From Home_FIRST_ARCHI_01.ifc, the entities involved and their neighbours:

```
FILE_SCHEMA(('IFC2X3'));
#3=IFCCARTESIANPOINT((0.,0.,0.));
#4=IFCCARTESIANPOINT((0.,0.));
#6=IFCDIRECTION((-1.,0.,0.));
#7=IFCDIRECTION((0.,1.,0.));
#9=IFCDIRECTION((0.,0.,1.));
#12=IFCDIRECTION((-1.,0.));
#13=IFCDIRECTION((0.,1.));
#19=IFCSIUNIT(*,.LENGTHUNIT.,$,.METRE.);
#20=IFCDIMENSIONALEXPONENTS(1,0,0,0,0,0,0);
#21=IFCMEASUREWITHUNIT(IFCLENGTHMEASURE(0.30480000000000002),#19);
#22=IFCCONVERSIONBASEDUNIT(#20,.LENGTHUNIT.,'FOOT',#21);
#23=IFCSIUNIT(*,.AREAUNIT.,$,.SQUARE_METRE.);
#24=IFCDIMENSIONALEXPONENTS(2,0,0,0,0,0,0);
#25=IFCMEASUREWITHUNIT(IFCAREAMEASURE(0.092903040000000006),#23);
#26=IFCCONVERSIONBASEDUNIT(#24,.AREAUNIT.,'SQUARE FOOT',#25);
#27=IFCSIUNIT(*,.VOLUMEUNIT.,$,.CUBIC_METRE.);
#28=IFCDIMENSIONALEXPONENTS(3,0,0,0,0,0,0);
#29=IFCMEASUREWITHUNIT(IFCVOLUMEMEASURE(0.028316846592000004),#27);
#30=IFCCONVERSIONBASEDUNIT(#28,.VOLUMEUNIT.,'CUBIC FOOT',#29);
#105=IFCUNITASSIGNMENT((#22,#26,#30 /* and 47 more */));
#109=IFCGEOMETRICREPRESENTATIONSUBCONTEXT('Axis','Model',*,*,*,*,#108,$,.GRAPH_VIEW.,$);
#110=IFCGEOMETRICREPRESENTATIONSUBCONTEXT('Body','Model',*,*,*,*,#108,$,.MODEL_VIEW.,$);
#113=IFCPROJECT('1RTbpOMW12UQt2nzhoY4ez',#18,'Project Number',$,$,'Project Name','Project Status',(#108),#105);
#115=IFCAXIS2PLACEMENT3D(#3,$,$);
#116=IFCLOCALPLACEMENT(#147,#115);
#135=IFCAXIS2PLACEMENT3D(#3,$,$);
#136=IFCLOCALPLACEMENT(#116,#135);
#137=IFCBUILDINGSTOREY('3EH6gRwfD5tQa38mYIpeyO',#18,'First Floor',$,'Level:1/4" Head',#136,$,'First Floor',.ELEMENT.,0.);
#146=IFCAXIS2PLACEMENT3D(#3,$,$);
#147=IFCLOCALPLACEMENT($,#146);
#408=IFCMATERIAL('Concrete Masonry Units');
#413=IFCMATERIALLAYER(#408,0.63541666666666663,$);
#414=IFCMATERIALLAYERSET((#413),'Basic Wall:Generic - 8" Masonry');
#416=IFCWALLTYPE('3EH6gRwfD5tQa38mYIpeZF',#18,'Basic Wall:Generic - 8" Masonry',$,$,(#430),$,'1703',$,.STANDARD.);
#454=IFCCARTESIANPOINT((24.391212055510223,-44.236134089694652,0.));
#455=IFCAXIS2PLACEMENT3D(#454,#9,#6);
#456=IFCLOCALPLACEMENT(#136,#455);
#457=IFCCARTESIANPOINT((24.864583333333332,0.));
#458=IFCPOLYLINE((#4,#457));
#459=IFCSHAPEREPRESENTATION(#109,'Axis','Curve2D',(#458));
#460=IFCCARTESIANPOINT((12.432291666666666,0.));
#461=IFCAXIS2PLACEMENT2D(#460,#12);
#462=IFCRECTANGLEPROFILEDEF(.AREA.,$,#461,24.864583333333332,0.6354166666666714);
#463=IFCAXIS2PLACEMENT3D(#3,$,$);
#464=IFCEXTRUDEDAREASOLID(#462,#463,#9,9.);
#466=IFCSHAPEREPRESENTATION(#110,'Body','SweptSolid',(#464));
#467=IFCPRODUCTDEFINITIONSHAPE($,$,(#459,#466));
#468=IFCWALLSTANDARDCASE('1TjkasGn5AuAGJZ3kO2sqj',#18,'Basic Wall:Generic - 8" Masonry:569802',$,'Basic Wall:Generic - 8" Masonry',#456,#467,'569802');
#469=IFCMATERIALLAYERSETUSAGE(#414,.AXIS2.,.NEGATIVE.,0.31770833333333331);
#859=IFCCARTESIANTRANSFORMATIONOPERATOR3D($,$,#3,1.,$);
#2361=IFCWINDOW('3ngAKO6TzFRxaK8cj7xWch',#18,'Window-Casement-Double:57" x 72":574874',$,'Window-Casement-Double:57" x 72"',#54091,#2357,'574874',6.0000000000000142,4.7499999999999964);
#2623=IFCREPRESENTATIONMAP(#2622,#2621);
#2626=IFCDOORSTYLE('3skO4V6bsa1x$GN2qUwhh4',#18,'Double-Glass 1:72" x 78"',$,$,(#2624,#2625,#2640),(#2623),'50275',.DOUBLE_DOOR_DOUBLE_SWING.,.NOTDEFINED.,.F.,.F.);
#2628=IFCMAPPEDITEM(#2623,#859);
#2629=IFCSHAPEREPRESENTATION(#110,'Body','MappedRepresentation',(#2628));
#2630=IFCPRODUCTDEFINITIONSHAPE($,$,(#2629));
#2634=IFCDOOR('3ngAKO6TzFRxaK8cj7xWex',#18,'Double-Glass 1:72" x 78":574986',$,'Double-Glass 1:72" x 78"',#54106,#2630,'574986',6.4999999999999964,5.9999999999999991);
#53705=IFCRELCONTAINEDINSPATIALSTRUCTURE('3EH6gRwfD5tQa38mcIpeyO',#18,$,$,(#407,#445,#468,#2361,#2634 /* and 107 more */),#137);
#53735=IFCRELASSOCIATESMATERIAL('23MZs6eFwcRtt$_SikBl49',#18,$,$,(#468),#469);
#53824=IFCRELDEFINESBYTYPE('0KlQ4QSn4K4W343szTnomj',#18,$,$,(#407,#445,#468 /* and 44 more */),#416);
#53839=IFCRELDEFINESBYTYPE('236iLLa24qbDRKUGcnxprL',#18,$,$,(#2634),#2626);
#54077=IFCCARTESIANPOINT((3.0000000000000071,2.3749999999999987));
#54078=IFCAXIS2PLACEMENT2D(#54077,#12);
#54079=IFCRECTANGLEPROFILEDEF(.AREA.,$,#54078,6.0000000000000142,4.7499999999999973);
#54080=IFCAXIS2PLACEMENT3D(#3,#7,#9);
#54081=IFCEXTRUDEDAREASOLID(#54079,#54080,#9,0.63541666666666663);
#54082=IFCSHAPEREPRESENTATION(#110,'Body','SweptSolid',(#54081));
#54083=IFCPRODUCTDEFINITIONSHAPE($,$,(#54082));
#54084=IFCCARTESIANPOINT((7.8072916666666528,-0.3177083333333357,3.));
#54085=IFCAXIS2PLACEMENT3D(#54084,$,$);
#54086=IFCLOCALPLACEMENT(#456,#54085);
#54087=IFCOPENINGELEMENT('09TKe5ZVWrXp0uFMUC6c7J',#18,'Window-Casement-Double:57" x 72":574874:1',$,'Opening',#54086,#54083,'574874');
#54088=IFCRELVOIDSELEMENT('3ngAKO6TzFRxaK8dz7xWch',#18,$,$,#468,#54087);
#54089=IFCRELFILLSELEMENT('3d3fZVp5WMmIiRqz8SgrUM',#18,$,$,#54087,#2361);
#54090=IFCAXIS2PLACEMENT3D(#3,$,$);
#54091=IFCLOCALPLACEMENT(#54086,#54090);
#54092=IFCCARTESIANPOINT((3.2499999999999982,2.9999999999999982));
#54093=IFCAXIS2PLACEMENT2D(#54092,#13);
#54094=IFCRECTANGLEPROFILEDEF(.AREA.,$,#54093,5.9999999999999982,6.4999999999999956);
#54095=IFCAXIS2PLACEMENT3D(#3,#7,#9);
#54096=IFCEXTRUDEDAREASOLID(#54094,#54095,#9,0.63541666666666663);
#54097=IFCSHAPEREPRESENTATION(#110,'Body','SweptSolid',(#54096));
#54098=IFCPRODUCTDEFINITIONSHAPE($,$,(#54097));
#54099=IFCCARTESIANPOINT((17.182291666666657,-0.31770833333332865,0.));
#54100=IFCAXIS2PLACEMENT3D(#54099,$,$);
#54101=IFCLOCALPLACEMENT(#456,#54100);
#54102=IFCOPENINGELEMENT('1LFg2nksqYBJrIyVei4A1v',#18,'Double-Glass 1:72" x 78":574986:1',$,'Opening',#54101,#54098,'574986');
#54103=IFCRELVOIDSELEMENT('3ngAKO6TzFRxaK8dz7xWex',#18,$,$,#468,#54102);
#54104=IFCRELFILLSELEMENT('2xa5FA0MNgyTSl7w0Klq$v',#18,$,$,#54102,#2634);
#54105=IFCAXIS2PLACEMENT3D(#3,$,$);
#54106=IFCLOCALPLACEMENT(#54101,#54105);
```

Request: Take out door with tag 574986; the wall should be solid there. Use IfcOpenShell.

```python
import ifcopenshell
import ifcopenshell.api.feature
import ifcopenshell.api.root
import ifcopenshell.geom
import ifcopenshell.util.shape

model = ifcopenshell.open("Home_FIRST_ARCHI_01.ifc")
settings = ifcopenshell.geom.settings()


def volume(element):
    """Net volume in cubic metres, openings subtracted."""
    shape = ifcopenshell.geom.create_shape(settings, element)
    return ifcopenshell.util.shape.get_volume(shape.geometry)


door = model.by_guid("3ngAKO6TzFRxaK8cj7xWex")
opening = door.FillsVoids[0].RelatingOpeningElement
wall = opening.VoidsElements[0].RelatingBuildingElement
before = volume(wall)

ifcopenshell.api.root.remove_product(model, product=door)
ifcopenshell.api.feature.remove_feature(model, feature=opening)

after = volume(wall)

print(f"wall volume {before:.3f} -> {after:.3f} m3")

model.write("Home_FIRST_ARCHI_01_edited.ifc")
```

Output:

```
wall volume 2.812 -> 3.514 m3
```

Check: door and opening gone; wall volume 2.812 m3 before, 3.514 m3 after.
